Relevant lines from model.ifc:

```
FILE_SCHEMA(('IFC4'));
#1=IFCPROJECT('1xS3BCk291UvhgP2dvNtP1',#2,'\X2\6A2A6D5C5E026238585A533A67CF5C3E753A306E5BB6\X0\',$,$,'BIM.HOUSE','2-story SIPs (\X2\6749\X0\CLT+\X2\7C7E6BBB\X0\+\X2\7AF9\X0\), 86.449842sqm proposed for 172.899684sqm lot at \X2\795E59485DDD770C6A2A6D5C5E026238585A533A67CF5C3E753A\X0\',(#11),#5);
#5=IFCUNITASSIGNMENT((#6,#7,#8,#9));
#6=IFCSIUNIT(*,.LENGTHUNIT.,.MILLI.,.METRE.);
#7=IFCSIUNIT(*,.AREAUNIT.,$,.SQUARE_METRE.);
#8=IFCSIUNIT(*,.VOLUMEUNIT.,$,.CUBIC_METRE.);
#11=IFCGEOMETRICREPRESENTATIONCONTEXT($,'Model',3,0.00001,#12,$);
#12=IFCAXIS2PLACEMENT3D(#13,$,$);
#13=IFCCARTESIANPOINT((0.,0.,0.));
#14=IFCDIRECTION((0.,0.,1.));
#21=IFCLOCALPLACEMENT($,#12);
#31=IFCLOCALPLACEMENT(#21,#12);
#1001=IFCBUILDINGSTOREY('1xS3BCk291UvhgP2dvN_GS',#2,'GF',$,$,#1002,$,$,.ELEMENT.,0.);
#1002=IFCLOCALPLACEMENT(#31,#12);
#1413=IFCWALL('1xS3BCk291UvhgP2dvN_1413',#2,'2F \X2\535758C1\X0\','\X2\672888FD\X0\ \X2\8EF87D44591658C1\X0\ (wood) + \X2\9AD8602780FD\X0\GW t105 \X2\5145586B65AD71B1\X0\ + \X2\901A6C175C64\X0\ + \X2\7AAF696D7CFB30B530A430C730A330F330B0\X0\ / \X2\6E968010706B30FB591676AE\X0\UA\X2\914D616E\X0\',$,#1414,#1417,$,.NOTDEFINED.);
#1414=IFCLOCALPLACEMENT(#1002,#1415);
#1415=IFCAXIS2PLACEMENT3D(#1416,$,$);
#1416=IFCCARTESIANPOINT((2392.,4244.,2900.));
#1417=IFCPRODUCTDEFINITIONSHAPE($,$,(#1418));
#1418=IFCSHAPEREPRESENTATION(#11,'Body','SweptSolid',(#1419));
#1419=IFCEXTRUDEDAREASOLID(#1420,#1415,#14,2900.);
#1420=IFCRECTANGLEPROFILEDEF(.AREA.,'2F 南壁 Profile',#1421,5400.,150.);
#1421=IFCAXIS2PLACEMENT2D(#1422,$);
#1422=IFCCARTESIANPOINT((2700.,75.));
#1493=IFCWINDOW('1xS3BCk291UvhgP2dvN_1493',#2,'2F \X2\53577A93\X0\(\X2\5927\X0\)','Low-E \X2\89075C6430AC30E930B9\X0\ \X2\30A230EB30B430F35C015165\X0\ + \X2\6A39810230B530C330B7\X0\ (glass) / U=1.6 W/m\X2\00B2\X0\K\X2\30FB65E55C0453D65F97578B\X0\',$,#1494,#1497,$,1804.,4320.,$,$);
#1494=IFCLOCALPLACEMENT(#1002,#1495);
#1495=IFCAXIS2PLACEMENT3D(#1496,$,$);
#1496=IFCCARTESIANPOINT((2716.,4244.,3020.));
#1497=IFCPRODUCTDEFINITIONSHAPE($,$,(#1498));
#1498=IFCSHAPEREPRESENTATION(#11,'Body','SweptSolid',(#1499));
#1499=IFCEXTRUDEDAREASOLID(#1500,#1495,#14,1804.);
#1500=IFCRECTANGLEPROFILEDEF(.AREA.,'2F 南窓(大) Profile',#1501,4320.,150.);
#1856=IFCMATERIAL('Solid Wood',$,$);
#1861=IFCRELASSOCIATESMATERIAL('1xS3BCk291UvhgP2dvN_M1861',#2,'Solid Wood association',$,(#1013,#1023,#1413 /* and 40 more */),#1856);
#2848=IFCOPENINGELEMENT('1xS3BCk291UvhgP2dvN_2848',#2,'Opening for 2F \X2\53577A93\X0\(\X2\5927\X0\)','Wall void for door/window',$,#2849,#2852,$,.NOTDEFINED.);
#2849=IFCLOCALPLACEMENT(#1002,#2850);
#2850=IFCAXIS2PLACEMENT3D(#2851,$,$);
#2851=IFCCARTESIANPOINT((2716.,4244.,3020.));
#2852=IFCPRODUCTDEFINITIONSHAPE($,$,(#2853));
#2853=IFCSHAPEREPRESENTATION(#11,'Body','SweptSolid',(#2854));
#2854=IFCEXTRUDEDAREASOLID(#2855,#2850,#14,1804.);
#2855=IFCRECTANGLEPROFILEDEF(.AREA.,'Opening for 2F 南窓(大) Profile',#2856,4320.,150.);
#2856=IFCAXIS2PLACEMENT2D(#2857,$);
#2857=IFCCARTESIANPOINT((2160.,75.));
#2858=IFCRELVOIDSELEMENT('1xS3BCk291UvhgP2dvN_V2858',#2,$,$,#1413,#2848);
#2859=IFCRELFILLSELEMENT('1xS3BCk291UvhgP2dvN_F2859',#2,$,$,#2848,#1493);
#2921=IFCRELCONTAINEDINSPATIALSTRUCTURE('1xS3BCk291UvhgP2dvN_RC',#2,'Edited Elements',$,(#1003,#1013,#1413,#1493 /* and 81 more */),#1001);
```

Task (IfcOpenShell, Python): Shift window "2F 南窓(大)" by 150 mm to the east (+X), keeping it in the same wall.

```python
import ifcopenshell
import ifcopenshell.api.geometry
import ifcopenshell.util.placement

model = ifcopenshell.open("model.ifc")

window = model.by_guid("1xS3BCk291UvhgP2dvN_1493")
opening = window.FillsVoids[0].RelatingOpeningElement
wall = opening.VoidsElements[0].RelatingBuildingElement

wall_matrix = ifcopenshell.util.placement.get_local_placement(wall.ObjectPlacement)
shift = wall_matrix[:3, 0] * 150.0
before = ifcopenshell.util.placement.get_local_placement(window.ObjectPlacement)[:3, 3].copy()

# The window is not placed relative to its opening, so move both.
for product in (opening, window):
    matrix = ifcopenshell.util.placement.get_local_placement(product.ObjectPlacement)
    matrix[:3, 3] += shift
    ifcopenshell.api.geometry.edit_object_placement(model, product=product, matrix=matrix, is_si=False)

after = ifcopenshell.util.placement.get_local_placement(window.ObjectPlacement)[:3, 3]
print("window moved by", (after - before).round(3) + 0.0)

model.write("model_updated.ifc")
```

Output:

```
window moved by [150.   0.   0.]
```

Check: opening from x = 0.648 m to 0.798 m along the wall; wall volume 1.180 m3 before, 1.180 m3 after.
